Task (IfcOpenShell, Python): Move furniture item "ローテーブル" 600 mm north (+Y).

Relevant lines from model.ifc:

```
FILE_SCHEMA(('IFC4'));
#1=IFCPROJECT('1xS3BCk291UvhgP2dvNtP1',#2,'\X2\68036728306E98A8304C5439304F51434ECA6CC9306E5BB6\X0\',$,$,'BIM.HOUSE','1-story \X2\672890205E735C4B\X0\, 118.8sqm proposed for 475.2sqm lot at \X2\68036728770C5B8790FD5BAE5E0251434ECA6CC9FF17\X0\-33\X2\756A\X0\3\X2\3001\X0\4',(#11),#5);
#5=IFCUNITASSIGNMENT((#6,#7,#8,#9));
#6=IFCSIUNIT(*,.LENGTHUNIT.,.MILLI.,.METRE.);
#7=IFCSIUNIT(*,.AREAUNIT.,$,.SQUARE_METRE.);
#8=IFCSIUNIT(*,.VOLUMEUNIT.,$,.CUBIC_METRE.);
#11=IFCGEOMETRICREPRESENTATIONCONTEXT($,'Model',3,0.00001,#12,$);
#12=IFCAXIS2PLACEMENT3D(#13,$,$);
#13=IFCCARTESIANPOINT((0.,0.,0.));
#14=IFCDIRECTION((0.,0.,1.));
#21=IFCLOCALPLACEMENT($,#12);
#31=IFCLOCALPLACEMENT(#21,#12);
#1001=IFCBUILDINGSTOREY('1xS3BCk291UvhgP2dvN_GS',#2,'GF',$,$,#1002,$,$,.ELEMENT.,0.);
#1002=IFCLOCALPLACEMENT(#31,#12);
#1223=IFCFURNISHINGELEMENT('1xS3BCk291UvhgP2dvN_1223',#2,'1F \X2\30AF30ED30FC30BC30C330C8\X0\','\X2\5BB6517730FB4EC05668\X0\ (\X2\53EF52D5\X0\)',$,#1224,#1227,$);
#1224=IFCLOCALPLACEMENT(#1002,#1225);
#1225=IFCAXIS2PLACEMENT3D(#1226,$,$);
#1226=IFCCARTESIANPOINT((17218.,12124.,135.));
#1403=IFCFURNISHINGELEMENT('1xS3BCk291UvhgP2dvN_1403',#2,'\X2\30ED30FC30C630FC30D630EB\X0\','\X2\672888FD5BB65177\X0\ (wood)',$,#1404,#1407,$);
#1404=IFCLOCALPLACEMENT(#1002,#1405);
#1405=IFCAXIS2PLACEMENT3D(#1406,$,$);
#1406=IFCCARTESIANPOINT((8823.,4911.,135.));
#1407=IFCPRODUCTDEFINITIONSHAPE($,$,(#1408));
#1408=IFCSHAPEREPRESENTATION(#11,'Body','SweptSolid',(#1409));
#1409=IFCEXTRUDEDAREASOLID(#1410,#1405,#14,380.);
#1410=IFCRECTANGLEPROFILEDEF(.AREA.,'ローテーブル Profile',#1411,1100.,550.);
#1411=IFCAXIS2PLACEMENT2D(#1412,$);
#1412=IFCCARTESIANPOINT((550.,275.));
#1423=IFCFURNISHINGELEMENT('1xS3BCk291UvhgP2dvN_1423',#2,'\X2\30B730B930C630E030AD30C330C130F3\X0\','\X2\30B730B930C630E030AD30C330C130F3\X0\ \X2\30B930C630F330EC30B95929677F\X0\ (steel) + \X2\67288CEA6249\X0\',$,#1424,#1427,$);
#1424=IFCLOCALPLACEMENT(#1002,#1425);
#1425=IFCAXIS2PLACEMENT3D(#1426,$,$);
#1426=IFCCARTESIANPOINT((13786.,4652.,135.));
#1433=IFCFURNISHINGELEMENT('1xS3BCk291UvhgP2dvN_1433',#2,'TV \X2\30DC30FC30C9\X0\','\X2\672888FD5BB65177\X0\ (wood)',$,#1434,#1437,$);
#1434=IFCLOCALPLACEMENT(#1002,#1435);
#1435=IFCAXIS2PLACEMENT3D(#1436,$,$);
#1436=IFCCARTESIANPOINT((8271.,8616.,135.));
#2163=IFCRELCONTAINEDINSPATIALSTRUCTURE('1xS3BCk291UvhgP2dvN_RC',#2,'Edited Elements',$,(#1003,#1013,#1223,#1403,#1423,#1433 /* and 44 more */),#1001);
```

```python
import ifcopenshell
import ifcopenshell.api.geometry
import ifcopenshell.util.placement

model = ifcopenshell.open("model.ifc")

item = model.by_guid("1xS3BCk291UvhgP2dvN_1403")
matrix = ifcopenshell.util.placement.get_local_placement(item.ObjectPlacement)
matrix[1, 3] += 600.0
ifcopenshell.api.geometry.edit_object_placement(model, product=item, matrix=matrix, is_si=False)

print(ifcopenshell.util.placement.get_local_placement(item.ObjectPlacement).round(3) + 0.0)

model.write("model_rev.ifc")
```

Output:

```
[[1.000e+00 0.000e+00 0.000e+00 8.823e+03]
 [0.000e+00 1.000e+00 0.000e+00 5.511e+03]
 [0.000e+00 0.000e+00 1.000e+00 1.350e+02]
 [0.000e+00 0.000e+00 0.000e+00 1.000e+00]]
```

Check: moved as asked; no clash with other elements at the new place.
